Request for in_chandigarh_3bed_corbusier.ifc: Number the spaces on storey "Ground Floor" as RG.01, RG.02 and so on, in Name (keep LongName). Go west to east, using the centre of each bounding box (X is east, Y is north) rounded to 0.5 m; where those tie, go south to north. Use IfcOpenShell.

First a look at what the model holds.

```python
import ifcopenshell
import ifcopenshell.util.element
import ifcopenshell.util.placement

model = ifcopenshell.open("in_chandigarh_3bed_corbusier.ifc")
print(model.schema)
storey = next(s for s in model.by_type("IfcBuildingStorey") if s.Name == "Ground Floor")
spaces = [e for e in ifcopenshell.util.element.get_decomposition(storey) if e.is_a("IfcSpace")]
for e in sorted(spaces, key=lambda e: e.id()):
    origin = ifcopenshell.util.placement.get_local_placement(e.ObjectPlacement)[:3, 3]
    print(e.id(), e.Name, e.LongName, origin.round(2) + 0.0, sep=" | ")
```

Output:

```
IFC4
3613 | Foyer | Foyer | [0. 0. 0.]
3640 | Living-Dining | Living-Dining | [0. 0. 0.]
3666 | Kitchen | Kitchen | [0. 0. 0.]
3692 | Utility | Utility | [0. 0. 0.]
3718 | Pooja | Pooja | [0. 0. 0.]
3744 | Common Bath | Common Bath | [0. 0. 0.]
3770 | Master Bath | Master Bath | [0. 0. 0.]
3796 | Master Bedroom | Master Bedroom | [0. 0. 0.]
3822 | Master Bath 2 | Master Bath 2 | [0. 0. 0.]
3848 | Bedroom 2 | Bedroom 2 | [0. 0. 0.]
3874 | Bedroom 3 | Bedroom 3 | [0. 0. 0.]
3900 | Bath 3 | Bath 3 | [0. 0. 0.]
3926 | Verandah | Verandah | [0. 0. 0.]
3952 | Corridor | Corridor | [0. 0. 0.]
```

```python
import ifcopenshell
import ifcopenshell.geom
import ifcopenshell.util.element
import ifcopenshell.util.shape

model = ifcopenshell.open("in_chandigarh_3bed_corbusier.ifc")
settings = ifcopenshell.geom.settings()
settings.set("use-world-coords", True)


def centre(element):
    shape = ifcopenshell.geom.create_shape(settings, element)
    return ifcopenshell.util.shape.get_bbox_centroid(shape.geometry)


storey = next(s for s in model.by_type("IfcBuildingStorey") if s.Name == "Ground Floor")
spaces = [e for e in ifcopenshell.util.element.get_decomposition(storey) if e.is_a("IfcSpace")]

# Insertion points can sit at a corner or the storey origin, so sort by the geometry (in metres).
centres = {e: centre(e) for e in spaces}
spaces.sort(key=lambda e: (round(centres[e][0] / 0.5), centres[e][1]))

for i, e in enumerate(spaces, start=1):
    number = f"RG.{i:02d}"
    e.Name = number
    print(e.id(), number)

model.write("in_chandigarh_3bed_corbusier-out.ifc")
```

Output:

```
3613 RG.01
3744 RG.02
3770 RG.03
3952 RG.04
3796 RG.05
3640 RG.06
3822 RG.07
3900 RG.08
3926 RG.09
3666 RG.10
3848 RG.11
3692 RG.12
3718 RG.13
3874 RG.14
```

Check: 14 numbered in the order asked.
